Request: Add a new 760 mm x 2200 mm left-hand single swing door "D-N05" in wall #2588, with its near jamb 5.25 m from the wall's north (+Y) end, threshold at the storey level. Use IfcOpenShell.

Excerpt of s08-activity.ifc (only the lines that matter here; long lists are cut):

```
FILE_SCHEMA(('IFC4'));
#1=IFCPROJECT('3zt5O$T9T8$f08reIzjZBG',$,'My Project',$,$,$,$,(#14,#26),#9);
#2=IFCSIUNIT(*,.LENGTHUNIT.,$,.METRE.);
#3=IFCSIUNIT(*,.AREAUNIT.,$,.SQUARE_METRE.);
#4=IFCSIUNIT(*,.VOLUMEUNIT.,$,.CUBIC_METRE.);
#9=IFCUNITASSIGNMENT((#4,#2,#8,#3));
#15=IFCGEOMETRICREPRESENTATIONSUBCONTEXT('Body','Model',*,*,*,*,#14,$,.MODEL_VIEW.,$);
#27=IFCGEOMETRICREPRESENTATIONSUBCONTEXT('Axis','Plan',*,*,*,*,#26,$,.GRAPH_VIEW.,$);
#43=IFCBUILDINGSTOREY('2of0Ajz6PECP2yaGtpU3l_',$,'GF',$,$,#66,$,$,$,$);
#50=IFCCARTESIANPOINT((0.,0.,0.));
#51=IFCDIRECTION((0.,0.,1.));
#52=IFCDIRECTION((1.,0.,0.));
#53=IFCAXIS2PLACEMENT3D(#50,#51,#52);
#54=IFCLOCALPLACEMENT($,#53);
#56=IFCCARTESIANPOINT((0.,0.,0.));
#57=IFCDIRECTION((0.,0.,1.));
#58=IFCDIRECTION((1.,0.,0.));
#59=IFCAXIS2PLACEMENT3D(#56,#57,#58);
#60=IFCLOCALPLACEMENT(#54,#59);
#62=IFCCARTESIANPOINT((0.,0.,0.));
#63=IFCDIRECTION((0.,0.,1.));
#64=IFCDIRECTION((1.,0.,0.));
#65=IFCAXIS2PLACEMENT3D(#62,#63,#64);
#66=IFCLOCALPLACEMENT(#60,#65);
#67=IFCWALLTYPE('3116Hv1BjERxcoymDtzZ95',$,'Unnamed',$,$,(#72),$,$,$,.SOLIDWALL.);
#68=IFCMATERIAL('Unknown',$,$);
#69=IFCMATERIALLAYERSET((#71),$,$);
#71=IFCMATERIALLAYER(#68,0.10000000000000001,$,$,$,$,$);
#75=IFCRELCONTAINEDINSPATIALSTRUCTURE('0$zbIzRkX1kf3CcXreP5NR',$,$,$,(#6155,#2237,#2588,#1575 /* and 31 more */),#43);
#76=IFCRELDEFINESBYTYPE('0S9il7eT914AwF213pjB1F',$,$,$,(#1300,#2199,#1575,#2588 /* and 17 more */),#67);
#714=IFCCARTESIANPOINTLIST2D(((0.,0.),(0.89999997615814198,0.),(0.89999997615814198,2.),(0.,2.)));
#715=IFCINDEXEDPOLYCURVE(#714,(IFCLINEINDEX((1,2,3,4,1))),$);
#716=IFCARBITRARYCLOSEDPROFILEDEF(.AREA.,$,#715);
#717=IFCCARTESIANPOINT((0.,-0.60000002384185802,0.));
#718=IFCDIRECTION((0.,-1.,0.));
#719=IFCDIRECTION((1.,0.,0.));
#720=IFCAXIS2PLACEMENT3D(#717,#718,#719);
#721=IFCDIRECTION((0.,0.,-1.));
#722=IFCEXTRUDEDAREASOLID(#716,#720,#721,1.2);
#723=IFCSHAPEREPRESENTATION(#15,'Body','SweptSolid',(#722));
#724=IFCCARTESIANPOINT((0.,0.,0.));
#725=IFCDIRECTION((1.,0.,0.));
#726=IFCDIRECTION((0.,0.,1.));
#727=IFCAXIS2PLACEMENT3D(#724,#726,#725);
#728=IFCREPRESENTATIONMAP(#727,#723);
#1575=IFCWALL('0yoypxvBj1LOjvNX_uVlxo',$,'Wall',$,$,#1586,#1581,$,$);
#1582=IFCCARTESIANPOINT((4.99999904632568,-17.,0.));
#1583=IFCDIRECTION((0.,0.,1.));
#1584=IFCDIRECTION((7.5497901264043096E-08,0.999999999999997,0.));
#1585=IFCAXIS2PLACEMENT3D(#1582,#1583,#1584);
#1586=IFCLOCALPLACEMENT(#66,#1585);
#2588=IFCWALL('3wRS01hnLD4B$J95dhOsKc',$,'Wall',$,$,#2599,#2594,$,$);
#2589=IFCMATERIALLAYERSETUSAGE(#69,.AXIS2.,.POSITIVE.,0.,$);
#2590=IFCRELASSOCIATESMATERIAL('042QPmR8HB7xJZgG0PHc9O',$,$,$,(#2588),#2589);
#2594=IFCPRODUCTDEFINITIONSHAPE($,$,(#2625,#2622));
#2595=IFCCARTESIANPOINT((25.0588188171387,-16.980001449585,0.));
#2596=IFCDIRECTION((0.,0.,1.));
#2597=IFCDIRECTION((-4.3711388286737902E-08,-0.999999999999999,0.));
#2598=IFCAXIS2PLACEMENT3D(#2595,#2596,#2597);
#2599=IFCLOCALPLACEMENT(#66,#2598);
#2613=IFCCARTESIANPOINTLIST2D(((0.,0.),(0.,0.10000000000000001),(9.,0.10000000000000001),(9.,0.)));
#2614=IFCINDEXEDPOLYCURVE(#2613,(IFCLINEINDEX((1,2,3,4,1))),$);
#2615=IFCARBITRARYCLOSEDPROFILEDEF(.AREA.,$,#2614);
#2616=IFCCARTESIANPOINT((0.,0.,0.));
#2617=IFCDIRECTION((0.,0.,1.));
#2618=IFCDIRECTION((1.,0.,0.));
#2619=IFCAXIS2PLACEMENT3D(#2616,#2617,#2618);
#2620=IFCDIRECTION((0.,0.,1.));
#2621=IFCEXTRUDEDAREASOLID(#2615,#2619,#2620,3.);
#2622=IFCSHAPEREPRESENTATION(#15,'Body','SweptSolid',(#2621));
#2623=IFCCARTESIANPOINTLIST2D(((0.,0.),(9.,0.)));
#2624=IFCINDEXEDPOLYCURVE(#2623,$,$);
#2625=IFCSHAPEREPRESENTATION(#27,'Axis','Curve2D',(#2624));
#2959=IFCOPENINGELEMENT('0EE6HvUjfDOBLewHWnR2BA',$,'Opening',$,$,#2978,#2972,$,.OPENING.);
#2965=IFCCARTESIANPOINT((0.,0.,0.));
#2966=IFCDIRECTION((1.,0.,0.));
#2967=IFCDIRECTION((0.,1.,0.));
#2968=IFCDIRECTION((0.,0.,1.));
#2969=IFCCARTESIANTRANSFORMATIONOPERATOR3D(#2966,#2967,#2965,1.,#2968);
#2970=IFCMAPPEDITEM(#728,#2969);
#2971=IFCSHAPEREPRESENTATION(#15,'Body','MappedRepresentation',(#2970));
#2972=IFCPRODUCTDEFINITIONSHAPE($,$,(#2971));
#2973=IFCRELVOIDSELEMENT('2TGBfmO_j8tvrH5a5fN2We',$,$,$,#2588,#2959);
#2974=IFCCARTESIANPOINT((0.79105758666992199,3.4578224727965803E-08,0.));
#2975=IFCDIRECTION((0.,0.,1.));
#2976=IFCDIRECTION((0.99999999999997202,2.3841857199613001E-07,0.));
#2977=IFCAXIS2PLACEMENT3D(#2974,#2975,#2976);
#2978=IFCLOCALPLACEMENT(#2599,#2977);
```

```python
import numpy as np
import ifcopenshell
import ifcopenshell.api.feature
import ifcopenshell.api.geometry
import ifcopenshell.api.root
import ifcopenshell.api.spatial
import ifcopenshell.geom
import ifcopenshell.util.element
import ifcopenshell.util.placement
import ifcopenshell.util.representation
import ifcopenshell.util.shape
import ifcopenshell.util.unit

model = ifcopenshell.open("s08-activity.ifc")
unit_scale = ifcopenshell.util.unit.calculate_unit_scale(model)
settings = ifcopenshell.geom.settings()


def volume(element):
    """Net volume in cubic metres, openings subtracted."""
    shape = ifcopenshell.geom.create_shape(settings, element)
    return ifcopenshell.util.shape.get_volume(shape.geometry)


wall = model.by_id(2588)
storey = ifcopenshell.util.element.get_container(wall, ifc_class="IfcBuildingStorey")
context = ifcopenshell.util.representation.get_context(model, "Model", "Body", "MODEL_VIEW")
before = volume(wall)

width, height, from_end, sill = 0.76, 2.2, 5.25, 0.0  # metres

# The wall runs along its own X axis, and the end named is its -X end.
wall_shape = ifcopenshell.geom.create_shape(settings, wall)
x, y, z = ifcopenshell.util.shape.get_vertices(wall_shape.geometry).T
start = x.min() + from_end
face, thickness = float(y.min()), float(y.max() - y.min())
wall_matrix = ifcopenshell.util.placement.get_local_placement(wall.ObjectPlacement)
level = ifcopenshell.util.placement.get_local_placement(storey.ObjectPlacement)[2, 3]


def in_wall(x, y):
    """Placement at x, y metres in the wall's axes, at sill height."""
    matrix = wall_matrix.copy()
    matrix[:, 3] = wall_matrix @ np.array([x / unit_scale, y / unit_scale, 0.0, 1.0])
    matrix[2, 3] = level + sill / unit_scale
    return matrix


# Opening: a box that overshoots both wall faces by 50 mm.
opening = ifcopenshell.api.root.create_entity(model, ifc_class="IfcOpeningElement", predefined_type="OPENING")
box = ifcopenshell.api.geometry.add_wall_representation(
    model, context=context, length=width, height=height, thickness=thickness + 0.1
)
ifcopenshell.api.geometry.assign_representation(model, product=opening, representation=box)
ifcopenshell.api.geometry.edit_object_placement(model, product=opening, matrix=in_wall(start, face - 0.05), is_si=False)
ifcopenshell.api.feature.add_feature(model, feature=opening, element=wall)

door = ifcopenshell.api.root.create_entity(model, ifc_class="IfcDoor", name="D-N05", predefined_type="DOOR")
door.OverallWidth, door.OverallHeight = width / unit_scale, height / unit_scale
door.OperationType = "SINGLE_SWING_LEFT"
body = ifcopenshell.api.geometry.add_door_representation(
    model,
    context=context,
    overall_width=door.OverallWidth,
    overall_height=door.OverallHeight,
    operation_type="SINGLE_SWING_LEFT",
    lining_properties={"LiningDepth": thickness / unit_scale, "ThresholdDepth": thickness / unit_scale},
)
ifcopenshell.api.geometry.assign_representation(model, product=door, representation=body)
ifcopenshell.api.spatial.assign_container(model, products=[door], relating_structure=storey)
ifcopenshell.api.feature.add_filling(model, opening=opening, element=door)

# The lining spans the wall, so the door starts at the wall face.
ifcopenshell.api.geometry.edit_object_placement(model, product=door, matrix=in_wall(start, face), is_si=False)

after = volume(wall)

print(f"wall volume {before:.3f} -> {after:.3f} m3")

model.write("s08-activity-out.ifc")
```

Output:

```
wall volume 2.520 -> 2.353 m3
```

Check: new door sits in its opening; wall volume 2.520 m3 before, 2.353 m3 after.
